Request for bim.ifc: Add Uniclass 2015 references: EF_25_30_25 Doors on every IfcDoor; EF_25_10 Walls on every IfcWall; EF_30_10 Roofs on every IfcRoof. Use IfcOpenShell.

First a look at what the model holds.

```python
import ifcopenshell

model = ifcopenshell.open("bim.ifc")
print(model.schema)
print("classifications:", [c.Name for c in model.by_type("IfcClassification")])
for ifc_class in ("IfcDoor", "IfcRoof", "IfcStair", "IfcWall", "IfcWindow"):
    print(ifc_class, len(model.by_type(ifc_class)))
```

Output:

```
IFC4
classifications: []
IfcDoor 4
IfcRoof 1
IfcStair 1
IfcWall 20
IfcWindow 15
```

```python
import ifcopenshell
import ifcopenshell.api.classification

model = ifcopenshell.open("bim.ifc")

system = ifcopenshell.api.classification.add_classification(model, classification="Uniclass 2015")

codes = {
    "IfcDoor": ("EF_25_30_25", "Doors"),
    "IfcWall": ("EF_25_10", "Walls"),
    "IfcRoof": ("EF_30_10", "Roofs"),
}
for ifc_class, (code, name) in codes.items():
    products = model.by_type(ifc_class)
    ifcopenshell.api.classification.add_reference(
        model, products=products, classification=system, identification=code, name=name
    )
    print(code, len(products))

model.write("bim_edited.ifc")
```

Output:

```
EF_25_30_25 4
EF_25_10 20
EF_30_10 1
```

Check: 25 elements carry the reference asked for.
